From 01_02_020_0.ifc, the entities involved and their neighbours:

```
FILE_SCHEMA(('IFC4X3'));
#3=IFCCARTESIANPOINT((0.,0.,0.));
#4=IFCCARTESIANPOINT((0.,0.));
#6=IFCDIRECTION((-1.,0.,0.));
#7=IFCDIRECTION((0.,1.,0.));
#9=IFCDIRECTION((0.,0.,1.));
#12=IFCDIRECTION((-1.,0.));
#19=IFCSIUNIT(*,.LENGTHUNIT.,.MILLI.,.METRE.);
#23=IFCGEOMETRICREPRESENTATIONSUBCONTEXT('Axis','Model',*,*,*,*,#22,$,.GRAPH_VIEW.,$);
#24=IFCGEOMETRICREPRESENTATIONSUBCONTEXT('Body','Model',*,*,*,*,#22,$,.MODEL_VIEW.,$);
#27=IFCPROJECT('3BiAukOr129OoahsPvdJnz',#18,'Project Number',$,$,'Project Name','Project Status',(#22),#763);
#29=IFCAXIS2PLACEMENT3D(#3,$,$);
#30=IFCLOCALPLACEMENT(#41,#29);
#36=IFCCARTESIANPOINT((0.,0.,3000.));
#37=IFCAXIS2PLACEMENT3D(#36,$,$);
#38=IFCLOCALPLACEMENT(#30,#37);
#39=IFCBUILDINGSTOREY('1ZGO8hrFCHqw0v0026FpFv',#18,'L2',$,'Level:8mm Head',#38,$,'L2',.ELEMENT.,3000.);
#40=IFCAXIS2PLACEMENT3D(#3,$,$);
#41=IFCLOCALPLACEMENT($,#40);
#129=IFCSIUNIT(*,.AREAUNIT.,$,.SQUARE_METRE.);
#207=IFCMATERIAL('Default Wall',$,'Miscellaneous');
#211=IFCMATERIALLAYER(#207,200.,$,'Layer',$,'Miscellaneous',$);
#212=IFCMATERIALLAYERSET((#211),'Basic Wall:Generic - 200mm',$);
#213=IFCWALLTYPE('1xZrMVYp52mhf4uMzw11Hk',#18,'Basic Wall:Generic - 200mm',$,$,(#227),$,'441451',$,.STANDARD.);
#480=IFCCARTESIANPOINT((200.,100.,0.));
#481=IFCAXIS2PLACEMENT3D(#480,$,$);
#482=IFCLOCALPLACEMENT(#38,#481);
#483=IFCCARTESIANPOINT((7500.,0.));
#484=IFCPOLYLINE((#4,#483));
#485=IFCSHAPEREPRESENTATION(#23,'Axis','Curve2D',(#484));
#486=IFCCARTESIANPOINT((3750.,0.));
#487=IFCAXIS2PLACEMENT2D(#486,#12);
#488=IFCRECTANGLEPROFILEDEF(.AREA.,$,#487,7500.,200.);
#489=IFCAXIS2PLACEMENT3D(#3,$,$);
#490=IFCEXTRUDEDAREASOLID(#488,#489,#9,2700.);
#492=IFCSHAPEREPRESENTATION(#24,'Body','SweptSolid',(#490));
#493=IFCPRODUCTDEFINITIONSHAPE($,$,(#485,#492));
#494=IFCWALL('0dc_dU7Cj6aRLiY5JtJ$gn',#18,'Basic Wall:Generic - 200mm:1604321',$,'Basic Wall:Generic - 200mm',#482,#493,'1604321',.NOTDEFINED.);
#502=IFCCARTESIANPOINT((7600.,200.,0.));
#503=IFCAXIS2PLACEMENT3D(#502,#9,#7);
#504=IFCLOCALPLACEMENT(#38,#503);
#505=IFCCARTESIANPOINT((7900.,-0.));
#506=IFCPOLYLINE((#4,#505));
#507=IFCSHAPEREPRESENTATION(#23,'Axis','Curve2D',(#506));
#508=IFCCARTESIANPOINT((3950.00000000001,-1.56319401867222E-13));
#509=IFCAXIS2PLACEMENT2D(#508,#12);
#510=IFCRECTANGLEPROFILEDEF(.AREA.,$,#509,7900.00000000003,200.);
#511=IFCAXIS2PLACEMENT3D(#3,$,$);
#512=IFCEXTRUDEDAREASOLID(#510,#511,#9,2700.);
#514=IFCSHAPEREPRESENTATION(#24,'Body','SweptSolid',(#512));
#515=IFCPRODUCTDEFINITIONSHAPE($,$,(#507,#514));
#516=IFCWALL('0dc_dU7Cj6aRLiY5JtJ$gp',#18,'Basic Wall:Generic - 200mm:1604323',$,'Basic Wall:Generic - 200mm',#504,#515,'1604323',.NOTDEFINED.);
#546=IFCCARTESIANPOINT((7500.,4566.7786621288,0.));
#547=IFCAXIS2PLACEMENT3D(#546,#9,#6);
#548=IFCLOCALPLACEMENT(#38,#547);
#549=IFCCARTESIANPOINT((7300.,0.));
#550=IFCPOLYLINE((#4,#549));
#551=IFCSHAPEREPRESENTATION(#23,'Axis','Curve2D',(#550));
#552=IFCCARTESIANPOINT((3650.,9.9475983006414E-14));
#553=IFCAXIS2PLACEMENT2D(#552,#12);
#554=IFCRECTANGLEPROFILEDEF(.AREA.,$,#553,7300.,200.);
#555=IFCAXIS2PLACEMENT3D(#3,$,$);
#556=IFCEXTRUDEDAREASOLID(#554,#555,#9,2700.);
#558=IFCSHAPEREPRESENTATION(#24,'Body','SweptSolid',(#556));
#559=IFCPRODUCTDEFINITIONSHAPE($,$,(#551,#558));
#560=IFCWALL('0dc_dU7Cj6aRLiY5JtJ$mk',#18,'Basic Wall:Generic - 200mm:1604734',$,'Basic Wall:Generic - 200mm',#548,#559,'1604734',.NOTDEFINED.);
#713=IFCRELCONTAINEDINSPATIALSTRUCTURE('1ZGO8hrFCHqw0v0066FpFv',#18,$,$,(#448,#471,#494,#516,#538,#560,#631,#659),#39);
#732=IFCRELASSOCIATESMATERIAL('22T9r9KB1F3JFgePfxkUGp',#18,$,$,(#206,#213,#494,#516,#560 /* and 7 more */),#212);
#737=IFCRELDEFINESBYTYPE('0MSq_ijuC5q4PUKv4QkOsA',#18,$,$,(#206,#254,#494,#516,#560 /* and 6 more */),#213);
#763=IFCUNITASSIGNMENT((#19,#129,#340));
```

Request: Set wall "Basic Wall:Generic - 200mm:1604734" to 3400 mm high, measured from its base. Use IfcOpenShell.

```python
import ifcopenshell
import ifcopenshell.geom
import ifcopenshell.util.representation
import ifcopenshell.util.shape

model = ifcopenshell.open("01_02_020_0.ifc")
settings = ifcopenshell.geom.settings()


def volume(element):
    """Net volume in cubic metres, openings subtracted."""
    shape = ifcopenshell.geom.create_shape(settings, element)
    return ifcopenshell.util.shape.get_volume(shape.geometry)


wall = model.by_guid("0dc_dU7Cj6aRLiY5JtJ$mk")
before = volume(wall)

body = ifcopenshell.util.representation.get_representation(wall, "Model", "Body")
solid = body.Items[0]
old_height = solid.Depth
solid.Depth = 3400.0
after = volume(wall)

print(f"height {old_height:g} -> {solid.Depth:g}, volume {before:.3f} -> {after:.3f} m3")

model.write("01_02_020_0-out.ifc")
```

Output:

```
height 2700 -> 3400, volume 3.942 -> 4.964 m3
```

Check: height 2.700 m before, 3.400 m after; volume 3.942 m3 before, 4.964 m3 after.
